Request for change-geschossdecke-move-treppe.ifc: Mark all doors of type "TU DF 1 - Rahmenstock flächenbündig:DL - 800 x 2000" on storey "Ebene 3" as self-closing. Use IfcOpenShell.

First a look at what the model holds.

```python
import ifcopenshell
import ifcopenshell.util.element

model = ifcopenshell.open("change-geschossdecke-move-treppe.ifc")
print(model.schema)
storey = next(s for s in model.by_type("IfcBuildingStorey") if s.Name == "Ebene 3")
doors = [e for e in ifcopenshell.util.element.get_decomposition(storey) if e.is_a("IfcDoor")]
seen = {}
for e in doors:
    element_type = ifcopenshell.util.element.get_type(e)
    key = (element_type.Name if element_type != e and element_type else None, ifcopenshell.util.element.get_pset(e, "Pset_DoorCommon", "SelfClosing"))
    seen[key] = seen.get(key, 0) + 1
for (name, value), count in sorted(seen.items(), key=str):
    print(count, "x", name, "|", value)
```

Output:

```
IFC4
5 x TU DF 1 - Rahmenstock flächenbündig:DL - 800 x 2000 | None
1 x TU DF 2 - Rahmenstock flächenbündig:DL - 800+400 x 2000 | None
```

```python
import ifcopenshell
import ifcopenshell.api.pset
import ifcopenshell.util.element

model = ifcopenshell.open("change-geschossdecke-move-treppe.ifc")

storey = next(s for s in model.by_type("IfcBuildingStorey") if s.Name == "Ebene 3")
doors = [e for e in ifcopenshell.util.element.get_decomposition(storey) if e.is_a("IfcDoor")]

count = 0
for e in doors:
    element_type = ifcopenshell.util.element.get_type(e)
    if element_type in (None, e) or element_type.Name != "TU DF 1 - Rahmenstock flächenbündig:DL - 800 x 2000":
        continue
    # add_pset returns the element's existing set when there is one.
    pset = ifcopenshell.api.pset.add_pset(model, product=e, name="Pset_DoorCommon")
    ifcopenshell.api.pset.edit_pset(model, pset=pset, properties={"SelfClosing": True})
    count += 1

print(count, "doors updated")

model.write("change-geschossdecke-move-treppe_v2.ifc")
```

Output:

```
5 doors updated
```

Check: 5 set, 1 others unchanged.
